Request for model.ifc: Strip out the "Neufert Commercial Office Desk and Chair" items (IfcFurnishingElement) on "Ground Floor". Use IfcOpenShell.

First a look at what the model holds.

```python
import ifcopenshell
import ifcopenshell.util.element

model = ifcopenshell.open("model.ifc")
print(model.schema)
storey = next(s for s in model.by_type("IfcBuildingStorey") if s.Name == "Ground Floor")
furniture = [e for e in ifcopenshell.util.element.get_decomposition(storey) if e.is_a("IfcFurnishingElement")]
seen = {}
for e in furniture:
    element_type = ifcopenshell.util.element.get_type(e)
    name = element_type.Name if element_type not in (None, e) else None
    seen[name] = seen.get(name, 0) + 1
for name, count in sorted(seen.items(), key=str):
    print(count, "x", name)
```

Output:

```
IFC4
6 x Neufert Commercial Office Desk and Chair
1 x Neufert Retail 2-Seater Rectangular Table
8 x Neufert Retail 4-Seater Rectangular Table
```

```python
import ifcopenshell
import ifcopenshell.api.root
import ifcopenshell.util.element

model = ifcopenshell.open("model.ifc")

storey = next(s for s in model.by_type("IfcBuildingStorey") if s.Name == "Ground Floor")
furniture = [e for e in ifcopenshell.util.element.get_decomposition(storey) if e.is_a("IfcFurnishingElement")]
targets = [e for e in furniture if (t := ifcopenshell.util.element.get_type(e)) not in (None, e) and t.Name == "Neufert Commercial Office Desk and Chair"]

for e in targets:
    ifcopenshell.api.root.remove_product(model, product=e)
print(len(targets), "removed")

model.write("model_edited.ifc")
```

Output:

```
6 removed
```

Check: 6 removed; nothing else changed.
